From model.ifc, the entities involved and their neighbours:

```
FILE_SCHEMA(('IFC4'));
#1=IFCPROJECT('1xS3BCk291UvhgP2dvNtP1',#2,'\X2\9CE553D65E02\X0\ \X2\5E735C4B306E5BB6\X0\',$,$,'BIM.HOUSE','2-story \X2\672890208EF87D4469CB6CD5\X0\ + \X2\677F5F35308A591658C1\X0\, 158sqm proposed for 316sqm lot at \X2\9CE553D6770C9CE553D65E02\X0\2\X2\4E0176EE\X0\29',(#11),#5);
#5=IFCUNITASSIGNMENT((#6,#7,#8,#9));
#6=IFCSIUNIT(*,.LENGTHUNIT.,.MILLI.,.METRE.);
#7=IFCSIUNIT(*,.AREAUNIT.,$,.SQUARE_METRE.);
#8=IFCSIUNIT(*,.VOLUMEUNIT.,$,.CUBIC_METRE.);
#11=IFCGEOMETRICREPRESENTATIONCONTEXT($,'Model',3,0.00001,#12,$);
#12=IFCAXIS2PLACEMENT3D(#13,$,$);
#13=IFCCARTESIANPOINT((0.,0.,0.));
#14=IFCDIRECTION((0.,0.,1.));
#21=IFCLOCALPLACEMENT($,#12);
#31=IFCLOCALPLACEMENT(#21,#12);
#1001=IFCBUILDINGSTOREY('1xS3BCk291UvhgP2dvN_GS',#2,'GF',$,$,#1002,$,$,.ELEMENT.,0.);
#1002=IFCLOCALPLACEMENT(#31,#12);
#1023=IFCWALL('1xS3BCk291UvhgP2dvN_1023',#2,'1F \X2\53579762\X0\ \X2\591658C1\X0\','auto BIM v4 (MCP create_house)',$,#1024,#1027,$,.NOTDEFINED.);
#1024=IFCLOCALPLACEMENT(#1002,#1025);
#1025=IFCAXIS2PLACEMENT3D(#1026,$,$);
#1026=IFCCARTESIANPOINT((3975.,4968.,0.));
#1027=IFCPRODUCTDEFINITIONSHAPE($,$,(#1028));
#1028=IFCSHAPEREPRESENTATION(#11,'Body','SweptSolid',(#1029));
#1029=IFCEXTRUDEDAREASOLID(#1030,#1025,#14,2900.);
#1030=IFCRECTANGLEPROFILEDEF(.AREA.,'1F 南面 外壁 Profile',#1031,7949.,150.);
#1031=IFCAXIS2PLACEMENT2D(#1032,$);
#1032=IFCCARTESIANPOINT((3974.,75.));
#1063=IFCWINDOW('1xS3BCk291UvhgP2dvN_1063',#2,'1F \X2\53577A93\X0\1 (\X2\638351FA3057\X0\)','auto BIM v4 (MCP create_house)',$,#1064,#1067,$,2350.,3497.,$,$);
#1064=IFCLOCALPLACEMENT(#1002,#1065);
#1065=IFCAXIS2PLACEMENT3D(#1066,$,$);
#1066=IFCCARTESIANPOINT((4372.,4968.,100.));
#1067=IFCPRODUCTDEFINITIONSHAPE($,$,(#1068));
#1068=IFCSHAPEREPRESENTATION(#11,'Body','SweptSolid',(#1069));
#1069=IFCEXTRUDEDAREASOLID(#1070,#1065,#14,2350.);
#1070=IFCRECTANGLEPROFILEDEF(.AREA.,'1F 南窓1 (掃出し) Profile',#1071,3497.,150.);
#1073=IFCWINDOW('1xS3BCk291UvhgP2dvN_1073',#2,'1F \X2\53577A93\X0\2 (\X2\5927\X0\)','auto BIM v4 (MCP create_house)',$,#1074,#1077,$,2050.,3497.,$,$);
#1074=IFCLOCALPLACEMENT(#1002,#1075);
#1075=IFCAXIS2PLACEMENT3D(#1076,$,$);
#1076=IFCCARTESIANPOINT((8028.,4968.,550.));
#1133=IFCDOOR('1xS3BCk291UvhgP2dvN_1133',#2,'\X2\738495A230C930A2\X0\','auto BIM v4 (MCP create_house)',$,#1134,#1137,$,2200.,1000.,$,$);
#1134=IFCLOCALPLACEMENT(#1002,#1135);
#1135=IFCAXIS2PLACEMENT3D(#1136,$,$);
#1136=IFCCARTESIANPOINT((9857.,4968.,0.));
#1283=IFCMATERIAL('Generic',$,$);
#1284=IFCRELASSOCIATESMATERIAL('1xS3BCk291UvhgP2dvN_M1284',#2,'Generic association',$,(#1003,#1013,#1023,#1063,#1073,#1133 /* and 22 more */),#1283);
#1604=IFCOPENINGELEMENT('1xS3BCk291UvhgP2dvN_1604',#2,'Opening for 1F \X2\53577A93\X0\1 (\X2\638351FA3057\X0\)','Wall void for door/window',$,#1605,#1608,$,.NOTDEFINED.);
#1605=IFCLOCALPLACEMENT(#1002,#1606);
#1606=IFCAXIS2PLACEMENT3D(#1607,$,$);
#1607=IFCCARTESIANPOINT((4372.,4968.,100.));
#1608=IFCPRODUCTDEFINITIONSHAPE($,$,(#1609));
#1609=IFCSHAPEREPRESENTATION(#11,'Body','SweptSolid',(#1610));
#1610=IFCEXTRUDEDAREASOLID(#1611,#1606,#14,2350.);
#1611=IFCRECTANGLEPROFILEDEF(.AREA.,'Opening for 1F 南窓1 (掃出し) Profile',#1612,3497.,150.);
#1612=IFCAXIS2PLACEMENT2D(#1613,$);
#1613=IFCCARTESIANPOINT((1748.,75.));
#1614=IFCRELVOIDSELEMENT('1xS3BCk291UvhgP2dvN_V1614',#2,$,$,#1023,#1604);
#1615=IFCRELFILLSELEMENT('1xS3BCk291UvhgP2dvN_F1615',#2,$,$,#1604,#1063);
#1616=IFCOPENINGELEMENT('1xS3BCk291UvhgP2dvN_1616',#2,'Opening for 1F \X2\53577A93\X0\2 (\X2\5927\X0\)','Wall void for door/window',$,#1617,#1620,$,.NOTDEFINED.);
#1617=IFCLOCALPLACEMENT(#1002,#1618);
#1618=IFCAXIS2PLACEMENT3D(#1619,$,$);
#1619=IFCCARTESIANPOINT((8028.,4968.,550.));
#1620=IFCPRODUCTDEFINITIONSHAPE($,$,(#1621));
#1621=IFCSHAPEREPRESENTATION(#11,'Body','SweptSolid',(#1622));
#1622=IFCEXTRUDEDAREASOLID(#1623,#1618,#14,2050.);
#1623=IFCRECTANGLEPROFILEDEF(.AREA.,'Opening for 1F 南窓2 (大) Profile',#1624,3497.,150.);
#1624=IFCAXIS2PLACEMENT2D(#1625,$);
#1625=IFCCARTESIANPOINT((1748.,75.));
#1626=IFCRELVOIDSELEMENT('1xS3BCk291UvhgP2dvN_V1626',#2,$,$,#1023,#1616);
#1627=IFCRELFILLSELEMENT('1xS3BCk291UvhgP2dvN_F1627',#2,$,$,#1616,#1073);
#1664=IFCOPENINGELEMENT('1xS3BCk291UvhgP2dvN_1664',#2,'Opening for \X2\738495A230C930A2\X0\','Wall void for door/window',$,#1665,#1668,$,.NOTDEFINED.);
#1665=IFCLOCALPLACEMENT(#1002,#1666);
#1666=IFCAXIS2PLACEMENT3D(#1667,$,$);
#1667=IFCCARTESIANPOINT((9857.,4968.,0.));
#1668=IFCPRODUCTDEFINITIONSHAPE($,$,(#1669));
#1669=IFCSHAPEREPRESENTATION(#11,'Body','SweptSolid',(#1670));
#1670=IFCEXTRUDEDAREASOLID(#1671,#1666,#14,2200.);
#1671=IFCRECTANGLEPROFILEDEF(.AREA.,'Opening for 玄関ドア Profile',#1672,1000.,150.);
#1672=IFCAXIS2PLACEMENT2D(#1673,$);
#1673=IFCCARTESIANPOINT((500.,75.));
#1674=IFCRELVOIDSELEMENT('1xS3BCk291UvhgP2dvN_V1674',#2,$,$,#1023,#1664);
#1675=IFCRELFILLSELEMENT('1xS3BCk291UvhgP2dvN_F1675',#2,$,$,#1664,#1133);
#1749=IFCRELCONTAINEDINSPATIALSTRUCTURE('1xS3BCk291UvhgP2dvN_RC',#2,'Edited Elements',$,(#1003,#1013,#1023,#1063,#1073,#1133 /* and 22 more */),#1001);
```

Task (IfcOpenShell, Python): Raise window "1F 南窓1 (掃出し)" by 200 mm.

```python
import numpy as np
import ifcopenshell
import ifcopenshell.api.geometry
import ifcopenshell.util.placement
import ifcopenshell.util.unit

model = ifcopenshell.open("model.ifc")
unit_scale = ifcopenshell.util.unit.calculate_unit_scale(model)

window = model.by_id(1063)
opening = window.FillsVoids[0].RelatingOpeningElement
dz = 0.2 / unit_scale

shift = np.array([0.0, 0.0, dz])
# The window is not placed relative to its opening, so move both.
for product in (opening, window):
    matrix = ifcopenshell.util.placement.get_local_placement(product.ObjectPlacement)
    matrix[:3, 3] += shift
    ifcopenshell.api.geometry.edit_object_placement(model, product=product, matrix=matrix, is_si=False)

print(f"moved by {dz * unit_scale:+.3f} m")

model.write("model_rev.ifc")
```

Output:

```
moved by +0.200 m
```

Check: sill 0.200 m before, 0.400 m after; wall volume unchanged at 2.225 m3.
